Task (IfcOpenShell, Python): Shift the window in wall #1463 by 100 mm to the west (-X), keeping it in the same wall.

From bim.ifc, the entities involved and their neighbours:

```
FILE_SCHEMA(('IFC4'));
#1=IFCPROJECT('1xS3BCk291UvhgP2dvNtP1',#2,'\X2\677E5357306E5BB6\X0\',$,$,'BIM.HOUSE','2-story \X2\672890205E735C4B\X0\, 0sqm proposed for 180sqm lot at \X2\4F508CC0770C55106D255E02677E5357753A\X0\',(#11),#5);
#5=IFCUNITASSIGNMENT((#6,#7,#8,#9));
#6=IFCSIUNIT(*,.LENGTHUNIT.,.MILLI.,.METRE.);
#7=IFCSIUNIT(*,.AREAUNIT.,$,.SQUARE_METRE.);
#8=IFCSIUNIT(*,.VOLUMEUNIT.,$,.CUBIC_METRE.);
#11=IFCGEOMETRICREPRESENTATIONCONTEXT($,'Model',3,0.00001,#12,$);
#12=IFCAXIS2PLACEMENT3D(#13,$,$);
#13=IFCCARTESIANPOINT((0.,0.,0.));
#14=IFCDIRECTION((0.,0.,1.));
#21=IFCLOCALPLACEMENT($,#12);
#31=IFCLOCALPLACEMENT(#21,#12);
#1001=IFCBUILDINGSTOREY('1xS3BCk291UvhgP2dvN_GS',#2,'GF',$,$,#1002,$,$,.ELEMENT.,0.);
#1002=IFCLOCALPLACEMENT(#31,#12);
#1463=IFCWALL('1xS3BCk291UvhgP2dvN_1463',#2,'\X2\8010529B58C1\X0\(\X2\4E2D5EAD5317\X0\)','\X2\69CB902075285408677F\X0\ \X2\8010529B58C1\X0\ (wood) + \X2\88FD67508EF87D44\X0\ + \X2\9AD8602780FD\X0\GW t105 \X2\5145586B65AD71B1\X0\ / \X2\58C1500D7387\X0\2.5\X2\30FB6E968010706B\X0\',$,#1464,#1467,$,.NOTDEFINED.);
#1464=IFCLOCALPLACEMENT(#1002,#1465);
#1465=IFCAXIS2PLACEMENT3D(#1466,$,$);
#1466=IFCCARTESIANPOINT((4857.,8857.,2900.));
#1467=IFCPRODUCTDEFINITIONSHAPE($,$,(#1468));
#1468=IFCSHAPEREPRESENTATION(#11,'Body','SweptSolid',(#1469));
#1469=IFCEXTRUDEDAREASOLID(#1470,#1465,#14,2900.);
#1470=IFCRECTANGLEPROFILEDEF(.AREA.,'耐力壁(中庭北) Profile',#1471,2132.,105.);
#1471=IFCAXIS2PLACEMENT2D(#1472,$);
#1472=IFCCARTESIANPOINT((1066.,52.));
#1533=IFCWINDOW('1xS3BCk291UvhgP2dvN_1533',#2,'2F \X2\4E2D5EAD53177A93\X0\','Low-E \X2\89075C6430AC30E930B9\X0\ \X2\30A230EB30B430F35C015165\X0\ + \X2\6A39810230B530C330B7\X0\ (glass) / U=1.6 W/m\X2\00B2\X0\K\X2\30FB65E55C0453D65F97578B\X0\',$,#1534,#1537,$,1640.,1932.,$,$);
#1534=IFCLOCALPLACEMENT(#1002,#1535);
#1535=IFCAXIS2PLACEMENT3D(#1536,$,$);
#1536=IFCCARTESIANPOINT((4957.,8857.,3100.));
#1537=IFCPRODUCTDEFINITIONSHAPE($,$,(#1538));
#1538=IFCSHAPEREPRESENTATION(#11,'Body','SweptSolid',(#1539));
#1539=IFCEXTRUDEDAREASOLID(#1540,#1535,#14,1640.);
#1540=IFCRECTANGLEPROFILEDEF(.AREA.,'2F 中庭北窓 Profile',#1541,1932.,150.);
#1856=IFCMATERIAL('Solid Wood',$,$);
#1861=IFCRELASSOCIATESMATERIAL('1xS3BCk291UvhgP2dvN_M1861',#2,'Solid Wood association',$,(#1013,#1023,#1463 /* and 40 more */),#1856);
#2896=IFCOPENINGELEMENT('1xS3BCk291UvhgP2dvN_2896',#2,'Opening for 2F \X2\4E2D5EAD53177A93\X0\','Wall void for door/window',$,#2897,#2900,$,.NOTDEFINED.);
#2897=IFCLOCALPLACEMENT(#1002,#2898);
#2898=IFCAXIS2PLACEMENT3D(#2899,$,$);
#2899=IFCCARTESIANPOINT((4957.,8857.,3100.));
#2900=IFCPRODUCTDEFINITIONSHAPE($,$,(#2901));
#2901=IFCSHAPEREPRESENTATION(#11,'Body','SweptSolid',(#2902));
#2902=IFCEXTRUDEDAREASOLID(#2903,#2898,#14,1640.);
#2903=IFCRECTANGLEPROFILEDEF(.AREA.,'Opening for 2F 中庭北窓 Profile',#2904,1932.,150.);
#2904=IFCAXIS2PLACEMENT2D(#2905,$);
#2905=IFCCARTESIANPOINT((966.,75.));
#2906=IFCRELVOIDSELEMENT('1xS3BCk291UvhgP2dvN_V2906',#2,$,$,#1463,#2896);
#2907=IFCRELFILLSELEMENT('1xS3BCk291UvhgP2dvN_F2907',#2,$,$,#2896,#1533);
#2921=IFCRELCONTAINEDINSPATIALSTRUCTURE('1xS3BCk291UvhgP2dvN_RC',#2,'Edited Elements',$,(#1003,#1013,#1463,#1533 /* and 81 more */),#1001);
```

```python
import ifcopenshell
import ifcopenshell.api.geometry
import ifcopenshell.util.placement

model = ifcopenshell.open("bim.ifc")

window = model.by_guid("1xS3BCk291UvhgP2dvN_1533")
opening = window.FillsVoids[0].RelatingOpeningElement
wall = opening.VoidsElements[0].RelatingBuildingElement

wall_matrix = ifcopenshell.util.placement.get_local_placement(wall.ObjectPlacement)
shift = wall_matrix[:3, 0] * -100.0
before = ifcopenshell.util.placement.get_local_placement(window.ObjectPlacement)[:3, 3].copy()

# The window is not placed relative to its opening, so move both.
for product in (opening, window):
    matrix = ifcopenshell.util.placement.get_local_placement(product.ObjectPlacement)
    matrix[:3, 3] += shift
    ifcopenshell.api.geometry.edit_object_placement(model, product=product, matrix=matrix, is_si=False)

after = ifcopenshell.util.placement.get_local_placement(window.ObjectPlacement)[:3, 3]
print("window moved by", (after - before).round(3) + 0.0)

model.write("bim_updated.ifc")
```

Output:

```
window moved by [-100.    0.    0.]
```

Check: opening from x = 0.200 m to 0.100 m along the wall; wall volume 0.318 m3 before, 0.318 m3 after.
